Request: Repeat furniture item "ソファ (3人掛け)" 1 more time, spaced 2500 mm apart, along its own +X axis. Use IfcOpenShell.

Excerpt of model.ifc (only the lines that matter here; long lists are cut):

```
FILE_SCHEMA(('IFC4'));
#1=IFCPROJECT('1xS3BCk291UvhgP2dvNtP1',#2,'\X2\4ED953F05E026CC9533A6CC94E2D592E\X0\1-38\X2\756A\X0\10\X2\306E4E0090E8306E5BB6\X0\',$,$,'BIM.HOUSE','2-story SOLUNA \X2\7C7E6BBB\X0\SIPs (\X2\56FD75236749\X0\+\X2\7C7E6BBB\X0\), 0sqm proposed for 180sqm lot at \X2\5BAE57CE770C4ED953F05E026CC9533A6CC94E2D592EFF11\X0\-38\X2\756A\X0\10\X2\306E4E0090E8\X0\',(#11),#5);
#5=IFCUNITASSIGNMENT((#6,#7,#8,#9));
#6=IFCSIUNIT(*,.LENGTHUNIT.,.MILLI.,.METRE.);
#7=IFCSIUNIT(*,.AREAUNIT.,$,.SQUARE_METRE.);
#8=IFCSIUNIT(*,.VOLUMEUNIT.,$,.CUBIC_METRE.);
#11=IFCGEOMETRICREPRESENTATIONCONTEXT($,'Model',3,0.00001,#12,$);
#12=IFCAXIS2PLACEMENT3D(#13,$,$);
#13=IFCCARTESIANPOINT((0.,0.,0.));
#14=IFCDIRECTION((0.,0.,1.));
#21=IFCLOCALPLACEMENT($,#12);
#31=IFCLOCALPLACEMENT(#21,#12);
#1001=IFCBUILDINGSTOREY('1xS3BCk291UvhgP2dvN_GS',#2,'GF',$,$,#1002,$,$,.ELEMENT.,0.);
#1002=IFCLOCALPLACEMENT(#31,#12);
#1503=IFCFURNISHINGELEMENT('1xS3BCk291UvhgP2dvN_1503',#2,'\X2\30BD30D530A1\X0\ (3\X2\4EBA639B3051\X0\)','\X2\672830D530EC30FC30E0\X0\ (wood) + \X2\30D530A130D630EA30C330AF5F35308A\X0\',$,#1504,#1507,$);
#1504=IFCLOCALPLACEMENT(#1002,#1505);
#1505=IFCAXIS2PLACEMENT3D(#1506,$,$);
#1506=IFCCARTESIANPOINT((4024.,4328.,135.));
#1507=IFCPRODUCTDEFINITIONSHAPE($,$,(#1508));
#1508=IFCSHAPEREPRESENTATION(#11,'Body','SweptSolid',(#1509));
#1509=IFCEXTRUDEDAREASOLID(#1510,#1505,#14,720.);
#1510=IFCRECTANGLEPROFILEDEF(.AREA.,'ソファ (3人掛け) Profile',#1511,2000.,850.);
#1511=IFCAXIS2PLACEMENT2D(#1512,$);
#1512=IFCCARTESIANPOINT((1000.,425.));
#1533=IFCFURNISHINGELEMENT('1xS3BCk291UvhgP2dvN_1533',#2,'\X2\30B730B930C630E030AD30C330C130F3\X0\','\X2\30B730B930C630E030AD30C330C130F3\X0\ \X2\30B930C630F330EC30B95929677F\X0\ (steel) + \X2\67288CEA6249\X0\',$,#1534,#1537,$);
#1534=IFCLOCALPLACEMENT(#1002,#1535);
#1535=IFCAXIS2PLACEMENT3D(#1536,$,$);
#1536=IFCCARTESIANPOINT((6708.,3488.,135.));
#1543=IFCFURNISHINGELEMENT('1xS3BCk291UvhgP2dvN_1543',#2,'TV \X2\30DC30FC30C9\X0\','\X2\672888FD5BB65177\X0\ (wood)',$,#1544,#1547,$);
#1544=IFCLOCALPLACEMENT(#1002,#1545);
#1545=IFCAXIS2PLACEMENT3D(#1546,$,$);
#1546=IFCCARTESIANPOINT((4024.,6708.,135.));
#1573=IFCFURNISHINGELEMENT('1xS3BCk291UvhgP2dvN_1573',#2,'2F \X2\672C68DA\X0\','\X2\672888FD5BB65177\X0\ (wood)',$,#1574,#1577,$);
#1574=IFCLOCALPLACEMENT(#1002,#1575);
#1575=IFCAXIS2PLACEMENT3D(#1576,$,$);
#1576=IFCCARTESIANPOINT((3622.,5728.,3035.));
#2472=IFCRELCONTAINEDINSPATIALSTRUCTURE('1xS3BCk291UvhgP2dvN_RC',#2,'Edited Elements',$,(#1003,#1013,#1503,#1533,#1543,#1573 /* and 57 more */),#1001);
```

```python
import ifcopenshell
import ifcopenshell.api.geometry
import ifcopenshell.api.root
import ifcopenshell.util.element
import ifcopenshell.util.placement
import ifcopenshell.util.unit

model = ifcopenshell.open("model.ifc")
unit_scale = ifcopenshell.util.unit.calculate_unit_scale(model)


def reuse_history(source, copy):
    """copy_class also copies each property set's owner history, people and application; keep the originals."""
    for rel in copy.IsDefinedBy:
        if rel.is_a("IfcRelDefinesByProperties") and (history := rel.RelatingPropertyDefinition.OwnerHistory):
            rel.RelatingPropertyDefinition.OwnerHistory = source.OwnerHistory
            ifcopenshell.util.element.remove_deep2(model, history)


source = model.by_id(1503)
base = ifcopenshell.util.placement.get_local_placement(source.ObjectPlacement)
step = base[:3, 0] * 2.5 / unit_scale

for i in range(1, 2):
    copy = ifcopenshell.api.root.copy_class(model, product=source)
    copy.Representation = ifcopenshell.util.element.copy_deep(
        model, source.Representation, exclude=["IfcGeometricRepresentationContext", "IfcRepresentationMap"]
    )
    reuse_history(source, copy)
    matrix = base.copy()
    matrix[:3, 3] += i * step
    print("added at", matrix[:3, 3].round(3) + 0.0)
    ifcopenshell.api.geometry.edit_object_placement(model, product=copy, matrix=matrix, is_si=False)

model.write("model_rev.ifc")
```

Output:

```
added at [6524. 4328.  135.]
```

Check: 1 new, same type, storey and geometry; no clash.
